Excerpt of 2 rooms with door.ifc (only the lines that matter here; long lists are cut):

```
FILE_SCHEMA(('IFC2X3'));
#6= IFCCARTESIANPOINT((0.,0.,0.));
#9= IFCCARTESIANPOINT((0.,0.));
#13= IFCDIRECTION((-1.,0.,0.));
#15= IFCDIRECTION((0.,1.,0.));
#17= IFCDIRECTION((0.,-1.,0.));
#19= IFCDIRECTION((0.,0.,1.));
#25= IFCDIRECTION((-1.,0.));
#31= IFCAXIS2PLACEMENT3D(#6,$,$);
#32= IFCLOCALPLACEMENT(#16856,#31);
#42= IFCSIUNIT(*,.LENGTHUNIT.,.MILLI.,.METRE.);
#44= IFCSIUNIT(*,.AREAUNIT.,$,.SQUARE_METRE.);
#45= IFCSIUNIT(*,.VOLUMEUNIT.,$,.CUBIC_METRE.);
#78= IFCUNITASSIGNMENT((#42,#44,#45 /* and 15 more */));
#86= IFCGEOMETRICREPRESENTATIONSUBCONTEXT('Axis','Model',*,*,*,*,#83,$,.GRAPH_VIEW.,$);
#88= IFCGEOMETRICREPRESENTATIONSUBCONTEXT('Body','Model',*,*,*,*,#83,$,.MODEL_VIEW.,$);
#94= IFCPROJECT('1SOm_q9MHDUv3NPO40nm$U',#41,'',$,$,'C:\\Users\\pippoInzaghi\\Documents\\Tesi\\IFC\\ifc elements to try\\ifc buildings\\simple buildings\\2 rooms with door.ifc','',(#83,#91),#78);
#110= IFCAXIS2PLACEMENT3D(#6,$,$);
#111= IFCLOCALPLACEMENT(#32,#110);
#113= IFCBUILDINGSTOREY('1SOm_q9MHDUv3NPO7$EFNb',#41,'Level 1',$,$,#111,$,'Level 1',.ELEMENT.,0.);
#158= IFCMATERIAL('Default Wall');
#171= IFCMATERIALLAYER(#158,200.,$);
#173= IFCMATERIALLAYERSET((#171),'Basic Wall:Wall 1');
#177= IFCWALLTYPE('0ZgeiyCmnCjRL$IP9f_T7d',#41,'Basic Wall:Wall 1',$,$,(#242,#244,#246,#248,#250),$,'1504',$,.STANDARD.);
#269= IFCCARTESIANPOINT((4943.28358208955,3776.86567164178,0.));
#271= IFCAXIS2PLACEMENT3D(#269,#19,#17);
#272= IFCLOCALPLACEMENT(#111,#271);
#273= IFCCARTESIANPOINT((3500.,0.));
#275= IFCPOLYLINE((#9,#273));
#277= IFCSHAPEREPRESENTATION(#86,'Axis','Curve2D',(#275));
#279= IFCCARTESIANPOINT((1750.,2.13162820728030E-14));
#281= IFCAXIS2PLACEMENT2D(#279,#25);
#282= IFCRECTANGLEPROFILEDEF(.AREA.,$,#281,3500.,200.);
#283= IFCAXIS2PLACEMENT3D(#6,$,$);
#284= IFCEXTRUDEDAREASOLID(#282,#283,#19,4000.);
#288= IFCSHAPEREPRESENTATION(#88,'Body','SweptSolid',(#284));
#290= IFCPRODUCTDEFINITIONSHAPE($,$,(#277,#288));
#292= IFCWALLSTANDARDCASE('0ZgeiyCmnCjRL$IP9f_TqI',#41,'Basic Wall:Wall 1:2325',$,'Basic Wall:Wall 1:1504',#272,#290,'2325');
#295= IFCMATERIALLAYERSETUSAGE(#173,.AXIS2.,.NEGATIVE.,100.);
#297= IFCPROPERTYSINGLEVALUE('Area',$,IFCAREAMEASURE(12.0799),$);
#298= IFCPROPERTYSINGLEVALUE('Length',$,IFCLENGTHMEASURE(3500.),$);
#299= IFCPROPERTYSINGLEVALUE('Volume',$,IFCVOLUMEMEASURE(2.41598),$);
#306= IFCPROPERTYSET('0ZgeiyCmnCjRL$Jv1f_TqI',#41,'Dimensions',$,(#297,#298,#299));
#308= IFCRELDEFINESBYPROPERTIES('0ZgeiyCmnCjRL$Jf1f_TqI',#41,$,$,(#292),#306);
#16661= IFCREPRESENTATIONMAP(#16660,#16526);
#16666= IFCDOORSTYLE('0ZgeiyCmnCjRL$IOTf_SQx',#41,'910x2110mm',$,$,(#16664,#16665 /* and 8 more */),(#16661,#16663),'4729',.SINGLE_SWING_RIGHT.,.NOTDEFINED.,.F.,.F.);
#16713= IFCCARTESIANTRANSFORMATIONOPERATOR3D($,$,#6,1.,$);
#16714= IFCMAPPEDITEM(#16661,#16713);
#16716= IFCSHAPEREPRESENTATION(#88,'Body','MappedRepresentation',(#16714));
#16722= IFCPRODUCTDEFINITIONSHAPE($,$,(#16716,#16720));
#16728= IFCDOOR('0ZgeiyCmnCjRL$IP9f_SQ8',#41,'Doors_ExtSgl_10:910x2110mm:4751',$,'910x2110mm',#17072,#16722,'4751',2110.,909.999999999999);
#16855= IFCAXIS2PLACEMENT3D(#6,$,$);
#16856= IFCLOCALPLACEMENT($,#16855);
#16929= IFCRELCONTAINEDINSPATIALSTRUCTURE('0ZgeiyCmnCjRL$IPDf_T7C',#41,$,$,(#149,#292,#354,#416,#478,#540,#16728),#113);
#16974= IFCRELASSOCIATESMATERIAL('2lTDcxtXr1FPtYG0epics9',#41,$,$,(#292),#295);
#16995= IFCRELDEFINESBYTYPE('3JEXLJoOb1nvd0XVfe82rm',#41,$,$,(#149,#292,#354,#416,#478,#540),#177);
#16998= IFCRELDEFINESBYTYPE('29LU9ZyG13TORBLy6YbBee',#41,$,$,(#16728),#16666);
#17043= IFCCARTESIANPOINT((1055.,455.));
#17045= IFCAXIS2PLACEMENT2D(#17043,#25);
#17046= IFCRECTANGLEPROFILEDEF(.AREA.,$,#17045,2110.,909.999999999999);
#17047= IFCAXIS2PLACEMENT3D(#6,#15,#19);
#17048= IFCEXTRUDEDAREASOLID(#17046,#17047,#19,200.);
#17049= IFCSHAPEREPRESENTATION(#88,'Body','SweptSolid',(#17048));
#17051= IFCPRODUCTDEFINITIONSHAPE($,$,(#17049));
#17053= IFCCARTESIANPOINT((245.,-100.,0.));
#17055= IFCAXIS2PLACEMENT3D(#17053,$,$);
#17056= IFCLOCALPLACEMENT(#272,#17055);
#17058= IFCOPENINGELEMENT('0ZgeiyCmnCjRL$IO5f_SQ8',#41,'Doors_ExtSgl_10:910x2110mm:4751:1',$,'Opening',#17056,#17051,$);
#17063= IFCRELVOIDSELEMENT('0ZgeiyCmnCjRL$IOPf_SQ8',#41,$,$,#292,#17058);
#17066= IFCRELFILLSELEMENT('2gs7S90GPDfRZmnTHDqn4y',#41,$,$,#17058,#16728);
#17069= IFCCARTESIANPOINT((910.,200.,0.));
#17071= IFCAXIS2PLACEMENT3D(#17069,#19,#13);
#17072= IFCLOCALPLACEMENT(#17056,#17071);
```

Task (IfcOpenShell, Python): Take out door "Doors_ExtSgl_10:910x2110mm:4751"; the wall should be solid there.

```python
import ifcopenshell
import ifcopenshell.api.feature
import ifcopenshell.api.pset
import ifcopenshell.api.root
import ifcopenshell.geom
import ifcopenshell.util.element
import ifcopenshell.util.shape
import ifcopenshell.util.unit

model = ifcopenshell.open("2 rooms with door.ifc")
area_scale = ifcopenshell.util.unit.calculate_unit_scale(model, "AREAUNIT")
volume_scale = ifcopenshell.util.unit.calculate_unit_scale(model, "VOLUMEUNIT")
settings = ifcopenshell.geom.settings()


def volume(element):
    """Net volume in cubic metres, openings subtracted."""
    shape = ifcopenshell.geom.create_shape(settings, element)
    return ifcopenshell.util.shape.get_volume(shape.geometry)


door = model.by_guid("0ZgeiyCmnCjRL$IP9f_SQ8")
opening = door.FillsVoids[0].RelatingOpeningElement
wall = opening.VoidsElements[0].RelatingBuildingElement
before = volume(wall)

ifcopenshell.api.root.remove_product(model, product=door)
ifcopenshell.api.feature.remove_feature(model, feature=opening)

after = volume(wall)
thickness = 0.2  # wall thickness in metres

# Update the wall's stored quantities.
pset = model.by_id(ifcopenshell.util.element.get_pset(wall, "Dimensions", should_inherit=False)["id"])
ifcopenshell.api.pset.edit_pset(model, pset=pset, properties={
    "Area": model.create_entity("IfcAreaMeasure", after / thickness / area_scale),
    "Volume": model.create_entity("IfcVolumeMeasure", after / volume_scale),
})

print(f"wall volume {before:.3f} -> {after:.3f} m3")

model.write("2 rooms with door_rev.ifc")
```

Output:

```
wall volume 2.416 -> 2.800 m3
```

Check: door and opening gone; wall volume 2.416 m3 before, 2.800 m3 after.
